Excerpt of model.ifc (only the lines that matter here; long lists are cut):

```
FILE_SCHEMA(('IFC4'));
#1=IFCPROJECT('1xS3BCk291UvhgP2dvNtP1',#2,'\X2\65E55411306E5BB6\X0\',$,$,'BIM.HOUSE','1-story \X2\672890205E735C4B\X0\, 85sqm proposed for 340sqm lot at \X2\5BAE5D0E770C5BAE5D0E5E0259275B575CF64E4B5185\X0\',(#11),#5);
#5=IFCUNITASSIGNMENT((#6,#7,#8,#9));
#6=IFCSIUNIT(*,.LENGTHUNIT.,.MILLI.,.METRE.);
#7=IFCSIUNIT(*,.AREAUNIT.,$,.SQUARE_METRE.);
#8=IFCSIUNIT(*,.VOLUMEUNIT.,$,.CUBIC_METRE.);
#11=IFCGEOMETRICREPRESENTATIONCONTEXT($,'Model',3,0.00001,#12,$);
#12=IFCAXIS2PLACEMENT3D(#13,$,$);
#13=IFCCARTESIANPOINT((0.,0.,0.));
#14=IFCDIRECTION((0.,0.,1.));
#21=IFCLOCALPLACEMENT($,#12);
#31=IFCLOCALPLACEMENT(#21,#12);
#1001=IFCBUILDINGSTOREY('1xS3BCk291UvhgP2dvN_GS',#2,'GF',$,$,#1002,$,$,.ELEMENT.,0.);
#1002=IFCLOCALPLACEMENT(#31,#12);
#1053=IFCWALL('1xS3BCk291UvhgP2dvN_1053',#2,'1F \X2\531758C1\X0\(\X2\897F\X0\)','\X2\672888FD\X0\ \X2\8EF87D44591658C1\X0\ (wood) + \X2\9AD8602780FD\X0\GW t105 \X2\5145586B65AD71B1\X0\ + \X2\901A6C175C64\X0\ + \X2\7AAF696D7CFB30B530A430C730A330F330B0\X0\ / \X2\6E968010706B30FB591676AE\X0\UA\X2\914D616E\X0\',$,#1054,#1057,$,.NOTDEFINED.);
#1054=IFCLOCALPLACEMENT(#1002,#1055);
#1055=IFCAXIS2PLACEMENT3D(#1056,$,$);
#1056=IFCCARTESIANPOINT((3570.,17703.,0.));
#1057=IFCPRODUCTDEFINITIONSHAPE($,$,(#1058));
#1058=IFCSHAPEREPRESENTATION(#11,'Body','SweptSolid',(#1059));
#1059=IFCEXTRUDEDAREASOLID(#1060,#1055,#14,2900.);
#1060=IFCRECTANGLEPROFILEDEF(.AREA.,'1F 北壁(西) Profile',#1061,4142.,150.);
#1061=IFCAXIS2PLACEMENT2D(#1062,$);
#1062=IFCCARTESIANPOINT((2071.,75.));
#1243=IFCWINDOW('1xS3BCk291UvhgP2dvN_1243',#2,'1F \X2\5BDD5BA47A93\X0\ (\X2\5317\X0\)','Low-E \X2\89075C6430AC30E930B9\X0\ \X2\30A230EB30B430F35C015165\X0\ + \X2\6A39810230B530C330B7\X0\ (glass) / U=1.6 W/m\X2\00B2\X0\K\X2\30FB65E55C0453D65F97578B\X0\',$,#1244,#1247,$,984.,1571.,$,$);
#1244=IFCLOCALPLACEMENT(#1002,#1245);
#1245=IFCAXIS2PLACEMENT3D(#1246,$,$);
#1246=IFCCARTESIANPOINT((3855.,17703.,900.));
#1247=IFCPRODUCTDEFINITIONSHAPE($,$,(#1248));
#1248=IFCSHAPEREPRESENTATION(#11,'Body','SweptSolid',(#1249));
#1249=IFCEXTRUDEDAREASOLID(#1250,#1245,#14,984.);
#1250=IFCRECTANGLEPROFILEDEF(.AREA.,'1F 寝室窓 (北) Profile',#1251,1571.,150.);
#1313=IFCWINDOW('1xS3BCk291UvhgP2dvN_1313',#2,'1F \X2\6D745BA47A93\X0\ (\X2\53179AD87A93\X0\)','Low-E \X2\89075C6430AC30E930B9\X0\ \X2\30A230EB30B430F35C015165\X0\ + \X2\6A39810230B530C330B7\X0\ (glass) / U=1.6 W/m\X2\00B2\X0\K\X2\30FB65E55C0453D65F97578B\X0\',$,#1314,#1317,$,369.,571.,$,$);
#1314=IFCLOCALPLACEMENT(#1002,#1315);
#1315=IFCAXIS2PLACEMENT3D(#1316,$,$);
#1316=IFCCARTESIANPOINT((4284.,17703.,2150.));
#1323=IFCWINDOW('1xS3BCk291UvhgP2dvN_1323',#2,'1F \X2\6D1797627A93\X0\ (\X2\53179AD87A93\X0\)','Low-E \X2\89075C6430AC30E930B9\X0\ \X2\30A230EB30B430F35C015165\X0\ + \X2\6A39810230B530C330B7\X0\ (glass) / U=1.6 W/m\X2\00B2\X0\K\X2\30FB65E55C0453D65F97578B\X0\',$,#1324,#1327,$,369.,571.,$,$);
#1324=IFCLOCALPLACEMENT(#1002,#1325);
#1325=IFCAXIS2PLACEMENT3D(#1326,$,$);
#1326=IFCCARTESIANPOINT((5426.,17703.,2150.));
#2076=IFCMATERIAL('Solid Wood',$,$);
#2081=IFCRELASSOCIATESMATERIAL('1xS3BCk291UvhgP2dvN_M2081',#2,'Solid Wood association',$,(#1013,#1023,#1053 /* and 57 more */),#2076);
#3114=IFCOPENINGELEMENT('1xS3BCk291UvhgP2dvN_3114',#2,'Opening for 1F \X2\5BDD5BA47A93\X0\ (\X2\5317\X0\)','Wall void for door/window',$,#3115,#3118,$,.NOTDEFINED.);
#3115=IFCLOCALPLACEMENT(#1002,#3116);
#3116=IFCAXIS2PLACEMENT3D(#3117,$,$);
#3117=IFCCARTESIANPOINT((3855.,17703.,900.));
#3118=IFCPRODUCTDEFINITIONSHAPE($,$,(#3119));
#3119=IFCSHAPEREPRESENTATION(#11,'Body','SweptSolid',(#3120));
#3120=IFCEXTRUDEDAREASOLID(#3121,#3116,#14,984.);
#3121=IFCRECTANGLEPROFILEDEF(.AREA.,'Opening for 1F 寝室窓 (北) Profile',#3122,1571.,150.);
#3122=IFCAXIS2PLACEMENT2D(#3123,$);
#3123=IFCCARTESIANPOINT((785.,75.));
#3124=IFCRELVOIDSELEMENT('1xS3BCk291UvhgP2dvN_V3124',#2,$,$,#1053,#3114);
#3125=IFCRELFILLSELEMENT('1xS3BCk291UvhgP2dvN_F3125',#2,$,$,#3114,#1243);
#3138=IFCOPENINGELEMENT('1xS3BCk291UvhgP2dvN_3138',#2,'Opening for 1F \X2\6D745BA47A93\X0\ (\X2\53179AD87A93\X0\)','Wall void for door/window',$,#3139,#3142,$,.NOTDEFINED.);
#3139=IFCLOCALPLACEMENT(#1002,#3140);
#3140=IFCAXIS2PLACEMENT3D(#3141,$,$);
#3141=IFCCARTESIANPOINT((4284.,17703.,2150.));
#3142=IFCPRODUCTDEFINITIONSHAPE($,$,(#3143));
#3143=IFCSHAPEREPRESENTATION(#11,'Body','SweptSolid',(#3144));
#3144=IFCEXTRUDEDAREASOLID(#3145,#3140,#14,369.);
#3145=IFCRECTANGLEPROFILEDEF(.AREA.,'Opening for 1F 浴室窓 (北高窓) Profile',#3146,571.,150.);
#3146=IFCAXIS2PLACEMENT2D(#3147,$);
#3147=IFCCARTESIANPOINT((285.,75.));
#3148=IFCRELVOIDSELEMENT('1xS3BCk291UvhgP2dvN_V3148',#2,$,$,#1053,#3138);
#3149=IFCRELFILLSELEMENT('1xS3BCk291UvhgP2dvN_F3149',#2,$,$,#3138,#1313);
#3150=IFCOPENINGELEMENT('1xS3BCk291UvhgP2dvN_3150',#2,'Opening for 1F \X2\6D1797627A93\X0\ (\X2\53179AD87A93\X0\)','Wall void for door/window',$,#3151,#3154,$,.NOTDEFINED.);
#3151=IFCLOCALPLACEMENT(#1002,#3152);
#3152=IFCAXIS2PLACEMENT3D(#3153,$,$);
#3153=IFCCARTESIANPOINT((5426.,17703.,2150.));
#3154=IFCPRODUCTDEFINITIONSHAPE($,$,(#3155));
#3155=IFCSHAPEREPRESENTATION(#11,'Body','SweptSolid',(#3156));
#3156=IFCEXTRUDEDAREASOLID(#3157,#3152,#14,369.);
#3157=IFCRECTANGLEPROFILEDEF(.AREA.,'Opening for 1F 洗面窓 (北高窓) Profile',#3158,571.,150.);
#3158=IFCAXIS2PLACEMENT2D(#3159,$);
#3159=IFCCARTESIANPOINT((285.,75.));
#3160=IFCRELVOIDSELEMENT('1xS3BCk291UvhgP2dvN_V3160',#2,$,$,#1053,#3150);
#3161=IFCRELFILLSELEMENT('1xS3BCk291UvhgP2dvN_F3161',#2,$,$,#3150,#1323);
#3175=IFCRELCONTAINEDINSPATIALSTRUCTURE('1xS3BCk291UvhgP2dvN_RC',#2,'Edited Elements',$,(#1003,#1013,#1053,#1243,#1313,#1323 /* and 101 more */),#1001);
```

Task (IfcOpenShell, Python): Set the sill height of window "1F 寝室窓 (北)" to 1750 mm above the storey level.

```python
import numpy as np
import ifcopenshell
import ifcopenshell.api.geometry
import ifcopenshell.geom
import ifcopenshell.util.element
import ifcopenshell.util.placement
import ifcopenshell.util.shape
import ifcopenshell.util.unit

model = ifcopenshell.open("model.ifc")
unit_scale = ifcopenshell.util.unit.calculate_unit_scale(model)

window = model.by_id(1243)
opening = window.FillsVoids[0].RelatingOpeningElement
storey = ifcopenshell.util.element.get_container(window, ifc_class="IfcBuildingStorey")
level = ifcopenshell.util.placement.get_local_placement(storey.ObjectPlacement)[2, 3]

# The opening's origin need not be at the sill, so measure its lowest point.
shape = ifcopenshell.geom.create_shape(ifcopenshell.geom.settings(), opening)
bottom = ifcopenshell.util.shape.get_shape_bottom_elevation(shape, shape.geometry) / unit_scale
dz = level + 1.75 / unit_scale - bottom

shift = np.array([0.0, 0.0, dz])
# The window is not placed relative to its opening, so move both.
for product in (opening, window):
    matrix = ifcopenshell.util.placement.get_local_placement(product.ObjectPlacement)
    matrix[:3, 3] += shift
    ifcopenshell.api.geometry.edit_object_placement(model, product=product, matrix=matrix, is_si=False)

print(f"moved by {dz * unit_scale:+.3f} m")

model.write("model-out.ifc")
```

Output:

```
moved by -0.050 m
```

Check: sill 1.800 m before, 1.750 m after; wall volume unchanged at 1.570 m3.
